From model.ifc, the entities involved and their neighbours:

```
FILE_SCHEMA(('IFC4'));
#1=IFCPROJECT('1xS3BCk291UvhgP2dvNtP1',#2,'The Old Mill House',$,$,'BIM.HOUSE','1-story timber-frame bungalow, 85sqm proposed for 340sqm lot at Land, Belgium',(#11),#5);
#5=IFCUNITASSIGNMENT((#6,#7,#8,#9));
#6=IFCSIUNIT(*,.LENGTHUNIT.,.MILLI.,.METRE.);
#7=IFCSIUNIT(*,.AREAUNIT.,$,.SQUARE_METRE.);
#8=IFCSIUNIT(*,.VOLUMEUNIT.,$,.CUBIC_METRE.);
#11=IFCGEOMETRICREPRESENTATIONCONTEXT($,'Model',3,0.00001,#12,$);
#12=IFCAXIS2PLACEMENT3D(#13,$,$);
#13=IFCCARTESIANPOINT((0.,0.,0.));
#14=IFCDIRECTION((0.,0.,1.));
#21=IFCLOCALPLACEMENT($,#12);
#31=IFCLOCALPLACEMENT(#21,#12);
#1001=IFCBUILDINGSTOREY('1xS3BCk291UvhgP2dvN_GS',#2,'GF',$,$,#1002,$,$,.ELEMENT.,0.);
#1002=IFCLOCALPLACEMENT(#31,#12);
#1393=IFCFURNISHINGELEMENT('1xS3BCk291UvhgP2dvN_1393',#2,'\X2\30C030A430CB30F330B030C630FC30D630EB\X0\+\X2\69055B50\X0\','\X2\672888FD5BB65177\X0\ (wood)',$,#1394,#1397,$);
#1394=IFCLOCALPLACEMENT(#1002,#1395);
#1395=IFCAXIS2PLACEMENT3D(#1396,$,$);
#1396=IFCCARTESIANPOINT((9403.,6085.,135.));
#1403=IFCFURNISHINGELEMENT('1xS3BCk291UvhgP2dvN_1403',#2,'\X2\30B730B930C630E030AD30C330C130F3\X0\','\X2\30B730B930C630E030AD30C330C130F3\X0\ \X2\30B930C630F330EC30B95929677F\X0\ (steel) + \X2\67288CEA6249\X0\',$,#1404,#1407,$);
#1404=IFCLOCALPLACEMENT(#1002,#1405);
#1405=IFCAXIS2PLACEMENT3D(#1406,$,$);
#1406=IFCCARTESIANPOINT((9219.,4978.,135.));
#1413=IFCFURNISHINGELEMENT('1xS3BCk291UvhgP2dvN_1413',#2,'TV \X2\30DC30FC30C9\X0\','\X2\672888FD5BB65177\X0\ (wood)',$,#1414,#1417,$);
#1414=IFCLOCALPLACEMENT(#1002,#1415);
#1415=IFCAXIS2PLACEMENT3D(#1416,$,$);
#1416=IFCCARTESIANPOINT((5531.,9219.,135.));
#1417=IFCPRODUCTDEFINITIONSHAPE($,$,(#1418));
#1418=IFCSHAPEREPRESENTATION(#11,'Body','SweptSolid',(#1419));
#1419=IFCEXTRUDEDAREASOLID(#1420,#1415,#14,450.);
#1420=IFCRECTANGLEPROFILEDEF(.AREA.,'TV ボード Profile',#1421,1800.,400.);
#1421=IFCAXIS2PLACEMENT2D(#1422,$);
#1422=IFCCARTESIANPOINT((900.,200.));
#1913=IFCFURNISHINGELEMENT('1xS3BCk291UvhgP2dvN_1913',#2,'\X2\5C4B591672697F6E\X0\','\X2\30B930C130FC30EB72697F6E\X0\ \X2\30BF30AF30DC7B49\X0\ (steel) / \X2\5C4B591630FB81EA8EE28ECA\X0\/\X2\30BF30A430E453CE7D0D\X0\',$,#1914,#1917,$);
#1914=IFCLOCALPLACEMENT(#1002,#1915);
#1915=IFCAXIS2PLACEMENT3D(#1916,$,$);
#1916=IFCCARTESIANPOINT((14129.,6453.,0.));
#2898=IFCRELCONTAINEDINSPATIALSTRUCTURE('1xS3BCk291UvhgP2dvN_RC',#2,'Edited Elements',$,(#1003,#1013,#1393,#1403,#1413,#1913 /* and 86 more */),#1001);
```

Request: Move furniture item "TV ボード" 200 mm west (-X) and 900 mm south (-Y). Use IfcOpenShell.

```python
import ifcopenshell
import ifcopenshell.api.geometry
import ifcopenshell.util.placement

model = ifcopenshell.open("model.ifc")

item = model.by_id(1413)
matrix = ifcopenshell.util.placement.get_local_placement(item.ObjectPlacement)
matrix[0, 3] -= 200.0
matrix[1, 3] -= 900.0
ifcopenshell.api.geometry.edit_object_placement(model, product=item, matrix=matrix, is_si=False)

print(ifcopenshell.util.placement.get_local_placement(item.ObjectPlacement).round(3) + 0.0)

model.write("model_v2.ifc")
```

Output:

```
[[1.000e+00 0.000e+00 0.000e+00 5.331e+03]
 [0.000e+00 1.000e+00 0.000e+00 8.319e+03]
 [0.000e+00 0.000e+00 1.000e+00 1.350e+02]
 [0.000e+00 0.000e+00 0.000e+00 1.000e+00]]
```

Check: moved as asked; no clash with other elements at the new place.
